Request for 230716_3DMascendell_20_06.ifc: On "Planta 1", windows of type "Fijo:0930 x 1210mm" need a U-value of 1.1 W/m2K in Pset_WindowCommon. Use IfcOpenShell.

First a look at what the model holds.

```python
import ifcopenshell
import ifcopenshell.util.element

model = ifcopenshell.open("230716_3DMascendell_20_06.ifc")
print(model.schema)
storey = next(s for s in model.by_type("IfcBuildingStorey") if s.Name == "Planta 1")
windows = [e for e in ifcopenshell.util.element.get_decomposition(storey) if e.is_a("IfcWindow")]
seen = {}
for e in windows:
    element_type = ifcopenshell.util.element.get_type(e)
    key = (element_type.Name if element_type != e and element_type else None, ifcopenshell.util.element.get_pset(e, "Pset_WindowCommon", "ThermalTransmittance"))
    seen[key] = seen.get(key, 0) + 1
for (name, value), count in sorted(seen.items(), key=str):
    print(count, "x", name, "|", value)
```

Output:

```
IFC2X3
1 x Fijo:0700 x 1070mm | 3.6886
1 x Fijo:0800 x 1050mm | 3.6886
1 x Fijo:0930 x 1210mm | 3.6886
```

```python
import ifcopenshell
import ifcopenshell.api.pset
import ifcopenshell.util.element

model = ifcopenshell.open("230716_3DMascendell_20_06.ifc")

storey = next(s for s in model.by_type("IfcBuildingStorey") if s.Name == "Planta 1")
windows = [e for e in ifcopenshell.util.element.get_decomposition(storey) if e.is_a("IfcWindow")]

count = 0
for e in windows:
    element_type = ifcopenshell.util.element.get_type(e)
    if element_type in (None, e) or element_type.Name != "Fijo:0930 x 1210mm":
        continue
    # add_pset returns the element's existing set when there is one.
    pset = ifcopenshell.api.pset.add_pset(model, product=e, name="Pset_WindowCommon")
    ifcopenshell.api.pset.edit_pset(model, pset=pset, properties={"ThermalTransmittance": 1.1})
    count += 1

print(count, "windows updated")

model.write("230716_3DMascendell_20_06_v2.ifc")
```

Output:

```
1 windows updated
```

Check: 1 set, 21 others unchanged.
